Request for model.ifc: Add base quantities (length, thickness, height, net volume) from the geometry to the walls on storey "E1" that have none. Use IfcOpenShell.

First a look at what the model holds.

```python
import ifcopenshell
import ifcopenshell.util.element
import ifcopenshell.util.unit

model = ifcopenshell.open("model.ifc")
print(model.schema)
for unit_type in ("LENGTHUNIT", "AREAUNIT", "VOLUMEUNIT"):
    print(unit_type, ifcopenshell.util.unit.calculate_unit_scale(model, unit_type))
storey = next(s for s in model.by_type("IfcBuildingStorey") if s.Name == "E1")
walls = [e for e in ifcopenshell.util.element.get_decomposition(storey) if e.is_a("IfcWall")]
for e in sorted(walls, key=lambda e: e.id()):
    print(e.id(), e.is_a(), e.Name, list(ifcopenshell.util.element.get_psets(e, qtos_only=True)), sep=" | ")
```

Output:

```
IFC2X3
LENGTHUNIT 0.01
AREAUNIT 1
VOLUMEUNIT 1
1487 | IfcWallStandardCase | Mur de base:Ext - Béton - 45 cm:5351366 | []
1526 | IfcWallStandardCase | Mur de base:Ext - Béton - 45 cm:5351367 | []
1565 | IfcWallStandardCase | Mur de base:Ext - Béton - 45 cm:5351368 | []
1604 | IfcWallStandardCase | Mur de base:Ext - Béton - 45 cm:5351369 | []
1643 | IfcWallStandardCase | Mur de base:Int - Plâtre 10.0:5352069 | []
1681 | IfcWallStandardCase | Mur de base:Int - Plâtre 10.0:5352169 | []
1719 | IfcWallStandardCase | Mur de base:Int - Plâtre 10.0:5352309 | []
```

```python
import ifcopenshell
import ifcopenshell.api.pset
import ifcopenshell.geom
import ifcopenshell.util.element
import ifcopenshell.util.shape
import ifcopenshell.util.unit

model = ifcopenshell.open("model.ifc")
unit_scale = ifcopenshell.util.unit.calculate_unit_scale(model)
volume_scale = ifcopenshell.util.unit.calculate_unit_scale(model, "VOLUMEUNIT")
settings = ifcopenshell.geom.settings()

storey = next(s for s in model.by_type("IfcBuildingStorey") if s.Name == "E1")
walls = [e for e in ifcopenshell.util.element.get_decomposition(storey) if e.is_a("IfcWall")]

for e in sorted(walls, key=lambda e: e.id()):
    if ifcopenshell.util.element.get_psets(e, qtos_only=True, should_inherit=False):
        continue
    # Geometry comes back in metres, in the element's own axes.
    shape = ifcopenshell.geom.create_shape(settings, e)
    values = {
        "Length": ifcopenshell.util.shape.get_x(shape.geometry) / unit_scale,
        "Width": ifcopenshell.util.shape.get_y(shape.geometry) / unit_scale,
        "Height": ifcopenshell.util.shape.get_z(shape.geometry) / unit_scale,
        "NetVolume": ifcopenshell.util.shape.get_volume(shape.geometry) / volume_scale,
    }
    qto = ifcopenshell.api.pset.add_qto(model, product=e, name="BaseQuantities")
    ifcopenshell.api.pset.edit_qto(model, qto=qto, properties=values)
    print(e.id(), {k: round(v, 3) for k, v in values.items()})

model.write("model_edited.ifc")
```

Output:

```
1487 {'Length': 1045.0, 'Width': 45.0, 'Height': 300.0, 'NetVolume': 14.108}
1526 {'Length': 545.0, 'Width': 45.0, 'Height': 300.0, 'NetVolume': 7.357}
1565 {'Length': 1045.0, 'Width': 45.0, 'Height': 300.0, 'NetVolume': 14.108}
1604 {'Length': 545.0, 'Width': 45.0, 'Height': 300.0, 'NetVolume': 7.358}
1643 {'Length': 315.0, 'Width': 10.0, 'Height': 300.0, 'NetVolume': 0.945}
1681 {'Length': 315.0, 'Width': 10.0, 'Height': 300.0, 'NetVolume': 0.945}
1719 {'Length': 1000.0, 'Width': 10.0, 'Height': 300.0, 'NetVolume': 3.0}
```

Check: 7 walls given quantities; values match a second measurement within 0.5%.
